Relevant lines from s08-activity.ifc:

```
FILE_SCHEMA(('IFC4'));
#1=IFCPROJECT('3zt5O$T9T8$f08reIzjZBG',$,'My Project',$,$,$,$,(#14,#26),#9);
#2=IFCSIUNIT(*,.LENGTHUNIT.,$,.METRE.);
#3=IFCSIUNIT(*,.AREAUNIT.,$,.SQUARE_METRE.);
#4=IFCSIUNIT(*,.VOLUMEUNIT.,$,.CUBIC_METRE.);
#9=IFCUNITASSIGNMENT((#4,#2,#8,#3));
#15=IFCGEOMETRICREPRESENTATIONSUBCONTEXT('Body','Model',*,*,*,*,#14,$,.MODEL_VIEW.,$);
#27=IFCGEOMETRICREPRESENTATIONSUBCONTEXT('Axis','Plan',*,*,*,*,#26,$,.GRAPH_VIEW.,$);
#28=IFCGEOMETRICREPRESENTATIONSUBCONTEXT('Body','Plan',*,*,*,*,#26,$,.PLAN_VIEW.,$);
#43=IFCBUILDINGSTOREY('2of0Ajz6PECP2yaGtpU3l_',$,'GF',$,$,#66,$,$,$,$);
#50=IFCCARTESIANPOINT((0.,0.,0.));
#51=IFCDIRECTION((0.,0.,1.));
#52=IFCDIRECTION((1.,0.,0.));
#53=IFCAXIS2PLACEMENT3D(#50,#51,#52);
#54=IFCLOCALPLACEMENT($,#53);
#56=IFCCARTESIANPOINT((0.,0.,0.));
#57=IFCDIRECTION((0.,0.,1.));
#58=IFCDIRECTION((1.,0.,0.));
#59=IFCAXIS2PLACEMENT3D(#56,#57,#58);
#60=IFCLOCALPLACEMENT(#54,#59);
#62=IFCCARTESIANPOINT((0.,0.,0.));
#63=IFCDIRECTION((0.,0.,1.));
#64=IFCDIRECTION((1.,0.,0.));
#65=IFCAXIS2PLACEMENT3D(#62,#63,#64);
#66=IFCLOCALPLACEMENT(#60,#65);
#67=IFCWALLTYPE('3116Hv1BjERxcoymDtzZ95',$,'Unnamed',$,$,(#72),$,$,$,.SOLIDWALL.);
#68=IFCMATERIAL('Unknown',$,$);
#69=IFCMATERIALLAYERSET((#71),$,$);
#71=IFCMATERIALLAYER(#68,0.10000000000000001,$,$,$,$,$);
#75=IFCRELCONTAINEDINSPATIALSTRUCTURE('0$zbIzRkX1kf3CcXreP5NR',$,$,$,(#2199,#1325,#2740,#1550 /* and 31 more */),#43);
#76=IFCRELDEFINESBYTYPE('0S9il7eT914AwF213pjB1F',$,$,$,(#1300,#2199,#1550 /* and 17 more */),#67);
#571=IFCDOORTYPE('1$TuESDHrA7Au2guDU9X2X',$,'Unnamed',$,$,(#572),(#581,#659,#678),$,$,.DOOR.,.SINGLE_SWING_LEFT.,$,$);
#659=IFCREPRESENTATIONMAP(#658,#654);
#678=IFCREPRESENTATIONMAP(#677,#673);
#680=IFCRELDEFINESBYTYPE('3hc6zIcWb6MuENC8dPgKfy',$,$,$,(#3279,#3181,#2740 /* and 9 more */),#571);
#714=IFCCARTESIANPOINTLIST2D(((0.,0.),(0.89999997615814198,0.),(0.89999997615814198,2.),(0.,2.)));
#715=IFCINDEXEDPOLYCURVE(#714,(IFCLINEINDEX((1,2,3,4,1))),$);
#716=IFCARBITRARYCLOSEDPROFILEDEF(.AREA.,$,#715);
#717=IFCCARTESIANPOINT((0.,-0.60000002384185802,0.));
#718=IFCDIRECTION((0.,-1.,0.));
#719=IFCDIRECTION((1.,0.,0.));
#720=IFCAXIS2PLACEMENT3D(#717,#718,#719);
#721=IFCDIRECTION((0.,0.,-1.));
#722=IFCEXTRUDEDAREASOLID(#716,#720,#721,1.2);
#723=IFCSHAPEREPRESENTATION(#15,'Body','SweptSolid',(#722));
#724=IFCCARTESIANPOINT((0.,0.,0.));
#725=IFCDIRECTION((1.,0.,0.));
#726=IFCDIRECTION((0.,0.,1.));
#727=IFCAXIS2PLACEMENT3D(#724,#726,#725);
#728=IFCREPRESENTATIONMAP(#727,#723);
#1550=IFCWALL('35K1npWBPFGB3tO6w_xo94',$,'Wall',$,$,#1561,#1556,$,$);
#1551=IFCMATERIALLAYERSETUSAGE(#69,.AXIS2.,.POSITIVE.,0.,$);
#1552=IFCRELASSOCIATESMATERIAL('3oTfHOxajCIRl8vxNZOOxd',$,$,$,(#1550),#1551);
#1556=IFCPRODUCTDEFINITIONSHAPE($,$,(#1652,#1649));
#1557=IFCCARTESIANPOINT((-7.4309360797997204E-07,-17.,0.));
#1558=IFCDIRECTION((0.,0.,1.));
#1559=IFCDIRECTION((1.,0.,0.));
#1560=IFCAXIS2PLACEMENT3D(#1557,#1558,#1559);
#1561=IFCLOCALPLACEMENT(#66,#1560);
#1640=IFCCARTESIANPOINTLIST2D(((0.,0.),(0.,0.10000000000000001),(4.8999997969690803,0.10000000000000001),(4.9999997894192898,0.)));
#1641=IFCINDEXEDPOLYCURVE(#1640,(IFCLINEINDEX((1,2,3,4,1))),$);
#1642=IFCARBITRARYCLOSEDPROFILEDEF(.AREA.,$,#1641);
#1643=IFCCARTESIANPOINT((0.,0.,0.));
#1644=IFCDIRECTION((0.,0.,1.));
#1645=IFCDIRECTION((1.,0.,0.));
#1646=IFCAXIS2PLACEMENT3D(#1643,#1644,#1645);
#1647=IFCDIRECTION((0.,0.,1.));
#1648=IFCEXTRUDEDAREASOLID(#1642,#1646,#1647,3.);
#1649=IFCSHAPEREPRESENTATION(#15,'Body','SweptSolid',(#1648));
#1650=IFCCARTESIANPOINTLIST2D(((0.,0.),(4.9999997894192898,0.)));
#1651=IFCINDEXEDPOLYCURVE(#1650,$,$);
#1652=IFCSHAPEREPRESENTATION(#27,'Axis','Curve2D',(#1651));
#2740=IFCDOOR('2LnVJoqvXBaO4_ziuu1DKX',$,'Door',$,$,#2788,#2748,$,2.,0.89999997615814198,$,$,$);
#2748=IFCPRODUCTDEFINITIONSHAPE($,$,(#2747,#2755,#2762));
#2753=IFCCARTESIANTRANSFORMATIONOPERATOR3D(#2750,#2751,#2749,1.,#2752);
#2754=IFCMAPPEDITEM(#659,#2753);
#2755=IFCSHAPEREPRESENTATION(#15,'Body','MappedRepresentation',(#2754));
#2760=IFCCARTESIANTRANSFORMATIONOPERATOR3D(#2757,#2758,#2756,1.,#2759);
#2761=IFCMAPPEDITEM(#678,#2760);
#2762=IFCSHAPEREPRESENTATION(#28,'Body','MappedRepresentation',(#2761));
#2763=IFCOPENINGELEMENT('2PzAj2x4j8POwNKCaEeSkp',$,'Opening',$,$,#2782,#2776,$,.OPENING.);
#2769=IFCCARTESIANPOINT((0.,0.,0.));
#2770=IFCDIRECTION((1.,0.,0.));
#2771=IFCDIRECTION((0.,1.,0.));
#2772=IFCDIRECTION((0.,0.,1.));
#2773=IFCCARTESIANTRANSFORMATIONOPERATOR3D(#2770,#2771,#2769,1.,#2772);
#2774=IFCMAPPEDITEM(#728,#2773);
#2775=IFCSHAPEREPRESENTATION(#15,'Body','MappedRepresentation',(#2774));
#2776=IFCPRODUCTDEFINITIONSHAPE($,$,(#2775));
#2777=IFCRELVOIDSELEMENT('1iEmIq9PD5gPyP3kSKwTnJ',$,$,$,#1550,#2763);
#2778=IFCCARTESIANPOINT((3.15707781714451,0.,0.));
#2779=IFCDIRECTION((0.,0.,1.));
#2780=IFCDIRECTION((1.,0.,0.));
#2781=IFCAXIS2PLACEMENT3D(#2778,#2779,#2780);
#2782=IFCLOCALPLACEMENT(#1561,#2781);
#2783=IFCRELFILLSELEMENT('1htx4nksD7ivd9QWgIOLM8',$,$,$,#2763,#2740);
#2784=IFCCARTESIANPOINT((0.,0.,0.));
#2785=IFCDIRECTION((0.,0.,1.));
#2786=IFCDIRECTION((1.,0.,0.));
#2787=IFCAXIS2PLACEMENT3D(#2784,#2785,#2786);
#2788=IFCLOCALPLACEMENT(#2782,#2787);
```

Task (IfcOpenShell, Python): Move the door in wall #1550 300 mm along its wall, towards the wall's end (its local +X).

```python
import ifcopenshell
import ifcopenshell.api.geometry
import ifcopenshell.util.placement

model = ifcopenshell.open("s08-activity.ifc")

door = model.by_id(2740)
opening = door.FillsVoids[0].RelatingOpeningElement
wall = opening.VoidsElements[0].RelatingBuildingElement

wall_matrix = ifcopenshell.util.placement.get_local_placement(wall.ObjectPlacement)
shift = wall_matrix[:3, 0] * 0.3
before = ifcopenshell.util.placement.get_local_placement(door.ObjectPlacement)[:3, 3].copy()

# The door is placed relative to its opening, so it follows when the opening moves.
matrix = ifcopenshell.util.placement.get_local_placement(opening.ObjectPlacement)
matrix[:3, 3] += shift
ifcopenshell.api.geometry.edit_object_placement(
    model, product=opening, matrix=matrix, is_si=False, should_transform_children=True
)

after = ifcopenshell.util.placement.get_local_placement(door.ObjectPlacement)[:3, 3]
print("door moved by", (after - before).round(3) + 0.0)

model.write("s08-activity_edited.ifc")
```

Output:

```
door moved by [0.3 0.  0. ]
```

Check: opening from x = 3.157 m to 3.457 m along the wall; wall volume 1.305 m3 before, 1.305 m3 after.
